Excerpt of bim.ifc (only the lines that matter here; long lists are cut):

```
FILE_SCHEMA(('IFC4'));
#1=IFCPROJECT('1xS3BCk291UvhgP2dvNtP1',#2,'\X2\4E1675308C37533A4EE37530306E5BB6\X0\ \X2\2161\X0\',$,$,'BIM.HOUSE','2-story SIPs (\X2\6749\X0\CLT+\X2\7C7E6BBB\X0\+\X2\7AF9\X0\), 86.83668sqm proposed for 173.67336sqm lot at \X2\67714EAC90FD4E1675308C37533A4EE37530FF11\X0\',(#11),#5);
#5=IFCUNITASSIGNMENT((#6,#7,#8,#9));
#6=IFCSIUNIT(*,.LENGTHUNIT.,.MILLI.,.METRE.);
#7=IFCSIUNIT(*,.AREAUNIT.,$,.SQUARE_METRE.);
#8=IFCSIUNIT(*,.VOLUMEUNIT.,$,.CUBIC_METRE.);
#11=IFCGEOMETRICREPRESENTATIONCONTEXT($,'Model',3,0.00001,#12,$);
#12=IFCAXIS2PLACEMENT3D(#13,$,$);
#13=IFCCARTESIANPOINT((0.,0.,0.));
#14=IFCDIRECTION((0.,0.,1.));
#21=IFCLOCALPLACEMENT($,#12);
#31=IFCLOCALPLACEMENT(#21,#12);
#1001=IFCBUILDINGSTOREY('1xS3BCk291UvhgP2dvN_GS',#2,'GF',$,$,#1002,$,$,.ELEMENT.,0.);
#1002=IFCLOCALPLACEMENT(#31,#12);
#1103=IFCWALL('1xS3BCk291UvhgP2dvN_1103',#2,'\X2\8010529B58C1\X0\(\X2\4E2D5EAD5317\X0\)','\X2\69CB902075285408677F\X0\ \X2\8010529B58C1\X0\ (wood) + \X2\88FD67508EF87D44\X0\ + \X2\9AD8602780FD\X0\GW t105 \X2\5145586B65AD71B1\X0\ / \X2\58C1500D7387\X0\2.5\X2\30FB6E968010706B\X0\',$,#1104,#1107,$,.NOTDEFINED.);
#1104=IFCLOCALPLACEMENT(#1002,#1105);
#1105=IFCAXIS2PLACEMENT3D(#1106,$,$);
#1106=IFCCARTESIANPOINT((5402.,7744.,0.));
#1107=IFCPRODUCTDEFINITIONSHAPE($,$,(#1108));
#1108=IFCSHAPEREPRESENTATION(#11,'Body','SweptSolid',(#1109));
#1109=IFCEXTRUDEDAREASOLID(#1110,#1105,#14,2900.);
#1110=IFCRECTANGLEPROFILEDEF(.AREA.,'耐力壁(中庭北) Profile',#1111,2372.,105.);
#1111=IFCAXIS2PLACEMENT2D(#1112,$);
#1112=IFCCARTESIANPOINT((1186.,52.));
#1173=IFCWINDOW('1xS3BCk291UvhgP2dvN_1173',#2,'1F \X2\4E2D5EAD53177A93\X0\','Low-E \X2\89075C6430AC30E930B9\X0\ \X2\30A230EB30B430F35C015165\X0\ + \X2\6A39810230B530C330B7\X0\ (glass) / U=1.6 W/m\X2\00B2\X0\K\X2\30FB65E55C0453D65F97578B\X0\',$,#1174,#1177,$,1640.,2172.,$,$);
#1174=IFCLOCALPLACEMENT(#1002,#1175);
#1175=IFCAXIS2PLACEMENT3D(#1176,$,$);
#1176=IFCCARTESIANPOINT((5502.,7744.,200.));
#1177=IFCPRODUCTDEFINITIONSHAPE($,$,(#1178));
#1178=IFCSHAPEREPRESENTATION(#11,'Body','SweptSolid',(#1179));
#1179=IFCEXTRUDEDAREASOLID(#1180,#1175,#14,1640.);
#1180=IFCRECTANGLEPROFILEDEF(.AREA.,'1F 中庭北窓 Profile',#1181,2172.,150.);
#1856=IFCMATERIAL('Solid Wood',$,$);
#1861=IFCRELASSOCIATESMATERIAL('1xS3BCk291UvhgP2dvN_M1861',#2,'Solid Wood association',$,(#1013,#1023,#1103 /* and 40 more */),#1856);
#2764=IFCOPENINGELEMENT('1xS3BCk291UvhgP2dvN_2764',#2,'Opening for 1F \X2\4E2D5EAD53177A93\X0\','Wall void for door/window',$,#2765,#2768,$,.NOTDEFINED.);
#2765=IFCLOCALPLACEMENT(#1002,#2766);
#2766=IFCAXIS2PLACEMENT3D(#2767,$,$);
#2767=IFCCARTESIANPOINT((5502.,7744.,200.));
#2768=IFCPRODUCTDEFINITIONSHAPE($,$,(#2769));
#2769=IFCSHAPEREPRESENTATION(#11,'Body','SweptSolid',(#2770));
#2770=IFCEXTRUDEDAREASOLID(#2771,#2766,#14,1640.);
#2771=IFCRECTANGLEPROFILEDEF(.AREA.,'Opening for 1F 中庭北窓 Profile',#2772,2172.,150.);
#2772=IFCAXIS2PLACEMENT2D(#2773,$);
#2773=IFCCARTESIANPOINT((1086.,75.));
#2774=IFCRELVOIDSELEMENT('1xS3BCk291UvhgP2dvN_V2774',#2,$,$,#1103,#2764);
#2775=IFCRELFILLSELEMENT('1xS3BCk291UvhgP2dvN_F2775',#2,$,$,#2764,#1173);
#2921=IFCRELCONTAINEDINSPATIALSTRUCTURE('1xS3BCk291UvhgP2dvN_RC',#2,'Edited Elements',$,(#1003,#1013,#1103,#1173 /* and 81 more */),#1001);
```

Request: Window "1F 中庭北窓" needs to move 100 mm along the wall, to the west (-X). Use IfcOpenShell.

```python
import ifcopenshell
import ifcopenshell.api.geometry
import ifcopenshell.util.placement
import ifcopenshell.util.unit

model = ifcopenshell.open("bim.ifc")
unit_scale = ifcopenshell.util.unit.calculate_unit_scale(model)

window = model.by_guid("1xS3BCk291UvhgP2dvN_1173")
opening = window.FillsVoids[0].RelatingOpeningElement
wall = opening.VoidsElements[0].RelatingBuildingElement

wall_matrix = ifcopenshell.util.placement.get_local_placement(wall.ObjectPlacement)
shift = wall_matrix[:3, 0] * -0.1 / unit_scale
before = ifcopenshell.util.placement.get_local_placement(window.ObjectPlacement)[:3, 3].copy()

# The window is not placed relative to its opening, so move both.
for product in (opening, window):
    matrix = ifcopenshell.util.placement.get_local_placement(product.ObjectPlacement)
    matrix[:3, 3] += shift
    ifcopenshell.api.geometry.edit_object_placement(model, product=product, matrix=matrix, is_si=False)

after = ifcopenshell.util.placement.get_local_placement(window.ObjectPlacement)[:3, 3]
print("window moved by", (after - before).round(3) + 0.0)

model.write("bim_v2.ifc")
```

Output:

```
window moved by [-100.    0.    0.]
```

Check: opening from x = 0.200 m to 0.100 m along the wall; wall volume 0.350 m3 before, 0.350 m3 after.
